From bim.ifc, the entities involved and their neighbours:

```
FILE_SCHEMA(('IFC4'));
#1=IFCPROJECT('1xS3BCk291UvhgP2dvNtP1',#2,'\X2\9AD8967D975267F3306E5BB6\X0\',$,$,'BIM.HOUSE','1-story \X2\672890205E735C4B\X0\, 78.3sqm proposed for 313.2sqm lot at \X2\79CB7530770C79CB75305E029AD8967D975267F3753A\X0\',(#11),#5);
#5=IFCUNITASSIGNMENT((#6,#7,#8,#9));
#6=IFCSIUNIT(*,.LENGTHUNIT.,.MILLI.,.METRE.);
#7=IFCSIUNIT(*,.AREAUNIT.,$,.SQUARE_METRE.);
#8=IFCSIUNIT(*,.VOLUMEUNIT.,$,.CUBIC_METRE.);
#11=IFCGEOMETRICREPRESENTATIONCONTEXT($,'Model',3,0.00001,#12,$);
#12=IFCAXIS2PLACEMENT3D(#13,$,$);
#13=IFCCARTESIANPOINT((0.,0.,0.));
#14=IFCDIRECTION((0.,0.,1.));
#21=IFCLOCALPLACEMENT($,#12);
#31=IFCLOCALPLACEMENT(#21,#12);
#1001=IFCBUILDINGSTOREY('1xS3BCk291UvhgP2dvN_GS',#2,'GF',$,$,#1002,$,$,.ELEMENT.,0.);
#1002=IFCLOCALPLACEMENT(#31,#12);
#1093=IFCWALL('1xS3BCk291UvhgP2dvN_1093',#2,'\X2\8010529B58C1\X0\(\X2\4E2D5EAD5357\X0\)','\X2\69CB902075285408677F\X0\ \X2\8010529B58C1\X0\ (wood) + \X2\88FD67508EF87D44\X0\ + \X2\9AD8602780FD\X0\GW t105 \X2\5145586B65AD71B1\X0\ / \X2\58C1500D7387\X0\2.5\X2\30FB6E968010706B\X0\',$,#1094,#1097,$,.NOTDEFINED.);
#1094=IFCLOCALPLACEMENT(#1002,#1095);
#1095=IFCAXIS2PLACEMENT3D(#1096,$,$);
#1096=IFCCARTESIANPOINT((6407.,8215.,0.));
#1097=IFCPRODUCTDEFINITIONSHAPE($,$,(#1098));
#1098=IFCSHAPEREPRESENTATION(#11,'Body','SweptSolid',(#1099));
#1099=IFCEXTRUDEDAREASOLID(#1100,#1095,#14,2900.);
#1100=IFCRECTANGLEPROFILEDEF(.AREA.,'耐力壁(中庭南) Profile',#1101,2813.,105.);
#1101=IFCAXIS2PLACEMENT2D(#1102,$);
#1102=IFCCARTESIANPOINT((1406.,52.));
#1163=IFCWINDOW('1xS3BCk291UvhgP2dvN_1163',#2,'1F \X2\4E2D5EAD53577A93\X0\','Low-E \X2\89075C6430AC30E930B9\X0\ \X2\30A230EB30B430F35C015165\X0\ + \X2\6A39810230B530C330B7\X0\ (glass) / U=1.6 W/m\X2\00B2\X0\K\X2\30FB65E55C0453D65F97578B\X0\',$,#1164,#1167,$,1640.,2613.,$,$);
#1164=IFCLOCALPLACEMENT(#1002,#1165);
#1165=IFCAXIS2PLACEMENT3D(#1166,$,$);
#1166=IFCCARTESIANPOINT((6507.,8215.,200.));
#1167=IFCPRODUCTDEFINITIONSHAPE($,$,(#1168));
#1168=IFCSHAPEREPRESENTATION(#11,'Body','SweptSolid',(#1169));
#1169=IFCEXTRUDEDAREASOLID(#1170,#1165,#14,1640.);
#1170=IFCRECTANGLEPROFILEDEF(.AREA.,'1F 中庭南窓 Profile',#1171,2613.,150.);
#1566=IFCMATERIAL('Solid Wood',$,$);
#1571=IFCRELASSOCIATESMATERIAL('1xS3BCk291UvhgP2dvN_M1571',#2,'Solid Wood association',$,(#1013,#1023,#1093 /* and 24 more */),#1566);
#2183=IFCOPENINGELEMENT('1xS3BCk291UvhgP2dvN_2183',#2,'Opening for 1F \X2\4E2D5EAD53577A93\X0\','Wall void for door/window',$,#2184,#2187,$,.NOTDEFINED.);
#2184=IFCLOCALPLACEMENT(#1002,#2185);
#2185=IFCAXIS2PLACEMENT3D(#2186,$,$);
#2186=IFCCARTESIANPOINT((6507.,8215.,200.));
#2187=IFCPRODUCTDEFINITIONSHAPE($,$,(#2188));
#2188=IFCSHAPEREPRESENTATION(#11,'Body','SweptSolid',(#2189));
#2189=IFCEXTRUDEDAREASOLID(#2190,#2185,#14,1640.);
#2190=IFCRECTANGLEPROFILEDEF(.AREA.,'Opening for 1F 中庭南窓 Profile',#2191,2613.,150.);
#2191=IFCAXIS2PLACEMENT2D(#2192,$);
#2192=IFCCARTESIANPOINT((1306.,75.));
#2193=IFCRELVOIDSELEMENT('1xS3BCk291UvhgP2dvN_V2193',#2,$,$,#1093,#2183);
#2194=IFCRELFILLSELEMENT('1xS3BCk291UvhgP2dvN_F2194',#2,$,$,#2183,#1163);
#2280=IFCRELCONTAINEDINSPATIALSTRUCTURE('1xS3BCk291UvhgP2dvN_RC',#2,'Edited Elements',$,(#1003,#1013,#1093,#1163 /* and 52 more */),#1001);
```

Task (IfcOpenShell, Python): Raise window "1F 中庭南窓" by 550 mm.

```python
import numpy as np
import ifcopenshell
import ifcopenshell.api.geometry
import ifcopenshell.util.placement
import ifcopenshell.util.unit

model = ifcopenshell.open("bim.ifc")
unit_scale = ifcopenshell.util.unit.calculate_unit_scale(model)

window = model.by_id(1163)
opening = window.FillsVoids[0].RelatingOpeningElement
dz = 0.55 / unit_scale

shift = np.array([0.0, 0.0, dz])
# The window is not placed relative to its opening, so move both.
for product in (opening, window):
    matrix = ifcopenshell.util.placement.get_local_placement(product.ObjectPlacement)
    matrix[:3, 3] += shift
    ifcopenshell.api.geometry.edit_object_placement(model, product=product, matrix=matrix, is_si=False)

print(f"moved by {dz * unit_scale:+.3f} m")

model.write("bim-out.ifc")
```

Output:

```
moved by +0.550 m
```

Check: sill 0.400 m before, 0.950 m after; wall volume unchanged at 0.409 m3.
